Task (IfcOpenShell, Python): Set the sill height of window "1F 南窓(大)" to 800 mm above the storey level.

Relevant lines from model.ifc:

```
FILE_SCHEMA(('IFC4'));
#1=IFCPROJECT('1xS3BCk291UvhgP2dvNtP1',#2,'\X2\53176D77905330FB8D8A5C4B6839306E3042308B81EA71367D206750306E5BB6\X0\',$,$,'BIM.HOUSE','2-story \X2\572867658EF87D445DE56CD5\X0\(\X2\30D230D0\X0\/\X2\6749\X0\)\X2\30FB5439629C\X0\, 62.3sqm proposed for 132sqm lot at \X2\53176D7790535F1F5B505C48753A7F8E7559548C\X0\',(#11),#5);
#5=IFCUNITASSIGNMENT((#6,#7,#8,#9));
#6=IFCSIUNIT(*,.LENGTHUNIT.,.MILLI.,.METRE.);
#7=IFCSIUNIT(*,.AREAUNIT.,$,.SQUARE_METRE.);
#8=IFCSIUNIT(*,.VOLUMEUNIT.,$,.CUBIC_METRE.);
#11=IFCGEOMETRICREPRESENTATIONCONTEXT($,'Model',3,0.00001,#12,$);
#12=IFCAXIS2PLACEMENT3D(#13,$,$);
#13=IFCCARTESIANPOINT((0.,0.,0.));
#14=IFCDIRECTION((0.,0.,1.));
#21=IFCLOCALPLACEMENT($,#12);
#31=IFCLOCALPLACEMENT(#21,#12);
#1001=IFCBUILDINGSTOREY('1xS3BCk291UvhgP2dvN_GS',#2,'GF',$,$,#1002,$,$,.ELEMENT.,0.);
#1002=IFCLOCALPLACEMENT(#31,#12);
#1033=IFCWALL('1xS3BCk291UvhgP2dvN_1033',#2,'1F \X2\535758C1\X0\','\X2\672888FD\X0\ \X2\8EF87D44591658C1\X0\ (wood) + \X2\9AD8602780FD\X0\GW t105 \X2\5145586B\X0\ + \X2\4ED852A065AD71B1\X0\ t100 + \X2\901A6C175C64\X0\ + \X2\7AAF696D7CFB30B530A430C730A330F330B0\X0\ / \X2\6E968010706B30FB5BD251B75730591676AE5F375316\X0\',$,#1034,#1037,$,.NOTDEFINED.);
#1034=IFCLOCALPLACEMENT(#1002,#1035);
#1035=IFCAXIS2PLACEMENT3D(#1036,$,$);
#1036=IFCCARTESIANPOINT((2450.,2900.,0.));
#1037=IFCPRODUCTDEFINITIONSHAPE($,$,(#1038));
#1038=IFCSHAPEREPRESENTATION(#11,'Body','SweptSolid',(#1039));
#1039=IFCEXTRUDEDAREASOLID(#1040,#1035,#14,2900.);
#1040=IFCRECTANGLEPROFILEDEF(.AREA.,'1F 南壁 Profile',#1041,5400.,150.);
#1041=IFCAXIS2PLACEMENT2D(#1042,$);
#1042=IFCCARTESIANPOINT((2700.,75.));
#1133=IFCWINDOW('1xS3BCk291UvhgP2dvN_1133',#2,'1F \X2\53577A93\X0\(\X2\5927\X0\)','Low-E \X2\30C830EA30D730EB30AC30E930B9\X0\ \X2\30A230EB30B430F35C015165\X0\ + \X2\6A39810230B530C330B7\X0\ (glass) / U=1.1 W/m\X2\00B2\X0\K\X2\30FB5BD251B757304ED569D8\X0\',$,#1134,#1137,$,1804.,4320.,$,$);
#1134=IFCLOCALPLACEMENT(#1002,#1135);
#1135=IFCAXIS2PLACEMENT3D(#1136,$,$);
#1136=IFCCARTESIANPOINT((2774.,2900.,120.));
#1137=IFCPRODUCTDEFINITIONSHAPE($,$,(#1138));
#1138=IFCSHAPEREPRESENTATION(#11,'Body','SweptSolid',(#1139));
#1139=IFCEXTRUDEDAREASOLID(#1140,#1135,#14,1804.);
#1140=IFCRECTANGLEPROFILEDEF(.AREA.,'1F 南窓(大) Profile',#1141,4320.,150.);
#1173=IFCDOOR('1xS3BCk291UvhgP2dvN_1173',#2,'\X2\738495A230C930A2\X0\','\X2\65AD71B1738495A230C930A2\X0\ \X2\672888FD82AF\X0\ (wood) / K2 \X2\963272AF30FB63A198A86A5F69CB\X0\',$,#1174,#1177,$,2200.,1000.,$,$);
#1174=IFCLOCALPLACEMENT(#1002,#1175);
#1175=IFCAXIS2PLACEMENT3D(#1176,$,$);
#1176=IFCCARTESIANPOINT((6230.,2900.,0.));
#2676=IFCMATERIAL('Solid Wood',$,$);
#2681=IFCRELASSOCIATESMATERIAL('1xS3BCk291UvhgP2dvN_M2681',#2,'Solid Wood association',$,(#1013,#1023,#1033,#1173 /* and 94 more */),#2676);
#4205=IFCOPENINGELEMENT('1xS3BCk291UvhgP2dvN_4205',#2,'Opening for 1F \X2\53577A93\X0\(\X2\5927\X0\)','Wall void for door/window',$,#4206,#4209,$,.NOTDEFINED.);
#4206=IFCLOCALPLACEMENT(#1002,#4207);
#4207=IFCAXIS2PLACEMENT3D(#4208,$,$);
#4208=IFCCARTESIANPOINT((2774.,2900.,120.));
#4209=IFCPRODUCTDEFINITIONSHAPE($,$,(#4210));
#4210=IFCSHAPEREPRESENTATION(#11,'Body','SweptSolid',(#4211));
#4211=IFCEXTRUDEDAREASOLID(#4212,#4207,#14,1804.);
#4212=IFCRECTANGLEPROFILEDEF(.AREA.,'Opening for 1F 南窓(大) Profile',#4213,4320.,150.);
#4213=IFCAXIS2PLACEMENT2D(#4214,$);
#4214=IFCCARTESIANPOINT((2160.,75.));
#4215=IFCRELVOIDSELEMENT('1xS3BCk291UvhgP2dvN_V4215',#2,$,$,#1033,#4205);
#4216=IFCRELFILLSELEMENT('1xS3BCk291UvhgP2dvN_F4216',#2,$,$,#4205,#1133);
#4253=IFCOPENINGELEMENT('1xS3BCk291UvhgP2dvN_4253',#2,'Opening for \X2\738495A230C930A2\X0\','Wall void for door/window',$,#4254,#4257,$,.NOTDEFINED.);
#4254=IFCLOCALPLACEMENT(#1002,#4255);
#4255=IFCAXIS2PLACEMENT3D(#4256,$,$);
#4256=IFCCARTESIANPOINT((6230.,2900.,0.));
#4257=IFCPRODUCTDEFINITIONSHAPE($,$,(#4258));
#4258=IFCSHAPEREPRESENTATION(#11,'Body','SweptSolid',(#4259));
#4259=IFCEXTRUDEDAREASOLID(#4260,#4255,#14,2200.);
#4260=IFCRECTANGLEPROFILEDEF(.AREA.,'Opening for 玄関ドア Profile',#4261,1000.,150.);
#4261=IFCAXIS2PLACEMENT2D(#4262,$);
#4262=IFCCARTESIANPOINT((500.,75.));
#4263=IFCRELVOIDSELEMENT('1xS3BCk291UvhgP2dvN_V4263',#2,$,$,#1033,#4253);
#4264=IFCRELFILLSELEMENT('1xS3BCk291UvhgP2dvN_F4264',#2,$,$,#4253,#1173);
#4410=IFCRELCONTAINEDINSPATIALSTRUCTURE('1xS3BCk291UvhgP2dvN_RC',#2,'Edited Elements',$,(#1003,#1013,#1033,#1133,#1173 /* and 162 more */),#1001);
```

```python
import numpy as np
import ifcopenshell
import ifcopenshell.api.geometry
import ifcopenshell.geom
import ifcopenshell.util.element
import ifcopenshell.util.placement
import ifcopenshell.util.shape
import ifcopenshell.util.unit

model = ifcopenshell.open("model.ifc")
unit_scale = ifcopenshell.util.unit.calculate_unit_scale(model)

window = model.by_id(1133)
opening = window.FillsVoids[0].RelatingOpeningElement
storey = ifcopenshell.util.element.get_container(window, ifc_class="IfcBuildingStorey")
level = ifcopenshell.util.placement.get_local_placement(storey.ObjectPlacement)[2, 3]

# The opening's origin need not be at the sill, so measure its lowest point.
shape = ifcopenshell.geom.create_shape(ifcopenshell.geom.settings(), opening)
bottom = ifcopenshell.util.shape.get_shape_bottom_elevation(shape, shape.geometry) / unit_scale
dz = level + 0.8 / unit_scale - bottom

shift = np.array([0.0, 0.0, dz])
# The window is not placed relative to its opening, so move both.
for product in (opening, window):
    matrix = ifcopenshell.util.placement.get_local_placement(product.ObjectPlacement)
    matrix[:3, 3] += shift
    ifcopenshell.api.geometry.edit_object_placement(model, product=product, matrix=matrix, is_si=False)

print(f"moved by {dz * unit_scale:+.3f} m")

model.write("model_edited.ifc")
```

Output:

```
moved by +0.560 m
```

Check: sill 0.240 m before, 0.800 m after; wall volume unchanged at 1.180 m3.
